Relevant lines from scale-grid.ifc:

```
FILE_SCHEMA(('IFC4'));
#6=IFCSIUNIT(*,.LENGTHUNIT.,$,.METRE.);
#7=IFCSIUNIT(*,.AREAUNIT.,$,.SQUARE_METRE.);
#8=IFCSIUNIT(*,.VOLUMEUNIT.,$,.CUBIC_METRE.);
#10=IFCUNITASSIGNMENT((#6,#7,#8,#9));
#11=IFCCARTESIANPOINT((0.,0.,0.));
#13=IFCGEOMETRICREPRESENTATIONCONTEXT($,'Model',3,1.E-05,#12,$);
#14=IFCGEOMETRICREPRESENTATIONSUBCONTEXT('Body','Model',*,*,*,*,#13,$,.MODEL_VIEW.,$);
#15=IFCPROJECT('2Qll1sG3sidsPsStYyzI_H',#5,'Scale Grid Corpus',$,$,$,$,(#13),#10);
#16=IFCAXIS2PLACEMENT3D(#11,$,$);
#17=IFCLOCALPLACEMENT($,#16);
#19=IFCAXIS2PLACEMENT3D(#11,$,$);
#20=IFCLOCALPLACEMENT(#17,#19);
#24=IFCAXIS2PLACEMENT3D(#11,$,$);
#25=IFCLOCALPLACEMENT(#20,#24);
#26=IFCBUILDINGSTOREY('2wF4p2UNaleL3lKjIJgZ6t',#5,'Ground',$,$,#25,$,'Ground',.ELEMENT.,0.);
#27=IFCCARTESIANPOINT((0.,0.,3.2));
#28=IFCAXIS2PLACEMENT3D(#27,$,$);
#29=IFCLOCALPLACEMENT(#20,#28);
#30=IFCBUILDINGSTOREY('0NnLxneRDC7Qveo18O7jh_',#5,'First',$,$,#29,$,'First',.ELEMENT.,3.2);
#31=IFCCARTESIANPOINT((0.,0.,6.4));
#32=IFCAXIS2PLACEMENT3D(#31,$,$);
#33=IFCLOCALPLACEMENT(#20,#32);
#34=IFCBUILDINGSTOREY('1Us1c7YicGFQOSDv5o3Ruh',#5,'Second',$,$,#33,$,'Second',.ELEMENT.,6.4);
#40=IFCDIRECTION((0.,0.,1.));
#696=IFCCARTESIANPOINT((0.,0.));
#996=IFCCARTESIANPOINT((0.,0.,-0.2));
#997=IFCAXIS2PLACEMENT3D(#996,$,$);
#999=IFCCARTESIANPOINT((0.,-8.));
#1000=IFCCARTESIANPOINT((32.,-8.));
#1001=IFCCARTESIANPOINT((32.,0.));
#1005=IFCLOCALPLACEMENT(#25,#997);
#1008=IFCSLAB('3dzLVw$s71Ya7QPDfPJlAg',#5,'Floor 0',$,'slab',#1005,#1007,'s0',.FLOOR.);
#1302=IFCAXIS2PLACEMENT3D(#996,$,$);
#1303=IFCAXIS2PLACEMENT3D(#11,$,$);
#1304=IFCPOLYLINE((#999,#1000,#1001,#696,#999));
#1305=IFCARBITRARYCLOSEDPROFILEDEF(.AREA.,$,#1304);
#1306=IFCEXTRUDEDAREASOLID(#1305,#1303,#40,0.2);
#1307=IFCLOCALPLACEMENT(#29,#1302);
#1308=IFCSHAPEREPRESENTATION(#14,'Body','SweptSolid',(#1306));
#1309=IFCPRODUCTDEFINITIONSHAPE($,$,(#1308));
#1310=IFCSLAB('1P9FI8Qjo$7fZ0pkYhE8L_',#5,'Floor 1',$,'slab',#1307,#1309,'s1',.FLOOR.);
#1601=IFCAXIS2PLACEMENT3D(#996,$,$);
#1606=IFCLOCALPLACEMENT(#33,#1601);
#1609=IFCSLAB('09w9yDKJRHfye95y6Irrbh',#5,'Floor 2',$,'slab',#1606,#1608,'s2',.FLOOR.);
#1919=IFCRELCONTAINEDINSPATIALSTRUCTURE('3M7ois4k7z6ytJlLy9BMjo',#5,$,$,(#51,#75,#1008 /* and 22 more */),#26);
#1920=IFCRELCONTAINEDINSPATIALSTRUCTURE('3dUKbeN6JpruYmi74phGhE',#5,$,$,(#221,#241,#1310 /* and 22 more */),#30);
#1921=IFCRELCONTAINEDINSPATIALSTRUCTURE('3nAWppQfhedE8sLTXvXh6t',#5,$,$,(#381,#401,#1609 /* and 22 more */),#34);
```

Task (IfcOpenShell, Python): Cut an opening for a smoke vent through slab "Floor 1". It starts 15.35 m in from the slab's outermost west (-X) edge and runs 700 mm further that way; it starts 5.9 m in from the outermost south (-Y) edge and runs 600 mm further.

```python
import numpy as np
import ifcopenshell
import ifcopenshell.api.feature
import ifcopenshell.api.geometry
import ifcopenshell.api.root
import ifcopenshell.geom
import ifcopenshell.util.placement
import ifcopenshell.util.representation
import ifcopenshell.util.shape
import ifcopenshell.util.unit

model = ifcopenshell.open("scale-grid.ifc")
unit_scale = ifcopenshell.util.unit.calculate_unit_scale(model)
settings = ifcopenshell.geom.settings()


def volume(element):
    """Net volume in cubic metres, openings subtracted."""
    shape = ifcopenshell.geom.create_shape(settings, element)
    return ifcopenshell.util.shape.get_volume(shape.geometry)


slab = model.by_guid("1P9FI8Qjo$7fZ0pkYhE8L_")
before = volume(slab)

# Extent in the slab's own axes, in metres. The edges named are its -X and -Y sides.
slab_shape = ifcopenshell.geom.create_shape(settings, slab)
vertices = ifcopenshell.util.shape.get_vertices(slab_shape.geometry)
x_min, y_min, bottom = vertices.min(axis=0)
top = vertices[:, 2].max()

opening = ifcopenshell.api.root.create_entity(model, ifc_class="IfcOpeningElement", name="Smoke vent opening", predefined_type="OPENING")
context = ifcopenshell.util.representation.get_context(model, "Model", "Body", "MODEL_VIEW")
width, depth = 0.7, 0.6
outline = [(0.0, 0.0), (width, 0.0), (width, depth), (0.0, depth), (0.0, 0.0)]
# Overshoot both faces by 50 mm so the cut is clean.
shape = ifcopenshell.api.geometry.add_slab_representation(
    model, context=context, depth=top - bottom + 0.1, polyline=outline
)
ifcopenshell.api.geometry.assign_representation(model, product=opening, representation=shape)

matrix = ifcopenshell.util.placement.get_local_placement(slab.ObjectPlacement)
matrix[:, 3] = matrix @ np.append(np.array([x_min + 15.35, y_min + 5.9, bottom - 0.05]) / unit_scale, 1.0)
ifcopenshell.api.geometry.edit_object_placement(model, product=opening, matrix=matrix, is_si=False)
ifcopenshell.api.feature.add_feature(model, feature=opening, element=slab)

after = volume(slab)

print(f"slab volume {before:.3f} -> {after:.3f} m3")

model.write("scale-grid_edited.ifc")
```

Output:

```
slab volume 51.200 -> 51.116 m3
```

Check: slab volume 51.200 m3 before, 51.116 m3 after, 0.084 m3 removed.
